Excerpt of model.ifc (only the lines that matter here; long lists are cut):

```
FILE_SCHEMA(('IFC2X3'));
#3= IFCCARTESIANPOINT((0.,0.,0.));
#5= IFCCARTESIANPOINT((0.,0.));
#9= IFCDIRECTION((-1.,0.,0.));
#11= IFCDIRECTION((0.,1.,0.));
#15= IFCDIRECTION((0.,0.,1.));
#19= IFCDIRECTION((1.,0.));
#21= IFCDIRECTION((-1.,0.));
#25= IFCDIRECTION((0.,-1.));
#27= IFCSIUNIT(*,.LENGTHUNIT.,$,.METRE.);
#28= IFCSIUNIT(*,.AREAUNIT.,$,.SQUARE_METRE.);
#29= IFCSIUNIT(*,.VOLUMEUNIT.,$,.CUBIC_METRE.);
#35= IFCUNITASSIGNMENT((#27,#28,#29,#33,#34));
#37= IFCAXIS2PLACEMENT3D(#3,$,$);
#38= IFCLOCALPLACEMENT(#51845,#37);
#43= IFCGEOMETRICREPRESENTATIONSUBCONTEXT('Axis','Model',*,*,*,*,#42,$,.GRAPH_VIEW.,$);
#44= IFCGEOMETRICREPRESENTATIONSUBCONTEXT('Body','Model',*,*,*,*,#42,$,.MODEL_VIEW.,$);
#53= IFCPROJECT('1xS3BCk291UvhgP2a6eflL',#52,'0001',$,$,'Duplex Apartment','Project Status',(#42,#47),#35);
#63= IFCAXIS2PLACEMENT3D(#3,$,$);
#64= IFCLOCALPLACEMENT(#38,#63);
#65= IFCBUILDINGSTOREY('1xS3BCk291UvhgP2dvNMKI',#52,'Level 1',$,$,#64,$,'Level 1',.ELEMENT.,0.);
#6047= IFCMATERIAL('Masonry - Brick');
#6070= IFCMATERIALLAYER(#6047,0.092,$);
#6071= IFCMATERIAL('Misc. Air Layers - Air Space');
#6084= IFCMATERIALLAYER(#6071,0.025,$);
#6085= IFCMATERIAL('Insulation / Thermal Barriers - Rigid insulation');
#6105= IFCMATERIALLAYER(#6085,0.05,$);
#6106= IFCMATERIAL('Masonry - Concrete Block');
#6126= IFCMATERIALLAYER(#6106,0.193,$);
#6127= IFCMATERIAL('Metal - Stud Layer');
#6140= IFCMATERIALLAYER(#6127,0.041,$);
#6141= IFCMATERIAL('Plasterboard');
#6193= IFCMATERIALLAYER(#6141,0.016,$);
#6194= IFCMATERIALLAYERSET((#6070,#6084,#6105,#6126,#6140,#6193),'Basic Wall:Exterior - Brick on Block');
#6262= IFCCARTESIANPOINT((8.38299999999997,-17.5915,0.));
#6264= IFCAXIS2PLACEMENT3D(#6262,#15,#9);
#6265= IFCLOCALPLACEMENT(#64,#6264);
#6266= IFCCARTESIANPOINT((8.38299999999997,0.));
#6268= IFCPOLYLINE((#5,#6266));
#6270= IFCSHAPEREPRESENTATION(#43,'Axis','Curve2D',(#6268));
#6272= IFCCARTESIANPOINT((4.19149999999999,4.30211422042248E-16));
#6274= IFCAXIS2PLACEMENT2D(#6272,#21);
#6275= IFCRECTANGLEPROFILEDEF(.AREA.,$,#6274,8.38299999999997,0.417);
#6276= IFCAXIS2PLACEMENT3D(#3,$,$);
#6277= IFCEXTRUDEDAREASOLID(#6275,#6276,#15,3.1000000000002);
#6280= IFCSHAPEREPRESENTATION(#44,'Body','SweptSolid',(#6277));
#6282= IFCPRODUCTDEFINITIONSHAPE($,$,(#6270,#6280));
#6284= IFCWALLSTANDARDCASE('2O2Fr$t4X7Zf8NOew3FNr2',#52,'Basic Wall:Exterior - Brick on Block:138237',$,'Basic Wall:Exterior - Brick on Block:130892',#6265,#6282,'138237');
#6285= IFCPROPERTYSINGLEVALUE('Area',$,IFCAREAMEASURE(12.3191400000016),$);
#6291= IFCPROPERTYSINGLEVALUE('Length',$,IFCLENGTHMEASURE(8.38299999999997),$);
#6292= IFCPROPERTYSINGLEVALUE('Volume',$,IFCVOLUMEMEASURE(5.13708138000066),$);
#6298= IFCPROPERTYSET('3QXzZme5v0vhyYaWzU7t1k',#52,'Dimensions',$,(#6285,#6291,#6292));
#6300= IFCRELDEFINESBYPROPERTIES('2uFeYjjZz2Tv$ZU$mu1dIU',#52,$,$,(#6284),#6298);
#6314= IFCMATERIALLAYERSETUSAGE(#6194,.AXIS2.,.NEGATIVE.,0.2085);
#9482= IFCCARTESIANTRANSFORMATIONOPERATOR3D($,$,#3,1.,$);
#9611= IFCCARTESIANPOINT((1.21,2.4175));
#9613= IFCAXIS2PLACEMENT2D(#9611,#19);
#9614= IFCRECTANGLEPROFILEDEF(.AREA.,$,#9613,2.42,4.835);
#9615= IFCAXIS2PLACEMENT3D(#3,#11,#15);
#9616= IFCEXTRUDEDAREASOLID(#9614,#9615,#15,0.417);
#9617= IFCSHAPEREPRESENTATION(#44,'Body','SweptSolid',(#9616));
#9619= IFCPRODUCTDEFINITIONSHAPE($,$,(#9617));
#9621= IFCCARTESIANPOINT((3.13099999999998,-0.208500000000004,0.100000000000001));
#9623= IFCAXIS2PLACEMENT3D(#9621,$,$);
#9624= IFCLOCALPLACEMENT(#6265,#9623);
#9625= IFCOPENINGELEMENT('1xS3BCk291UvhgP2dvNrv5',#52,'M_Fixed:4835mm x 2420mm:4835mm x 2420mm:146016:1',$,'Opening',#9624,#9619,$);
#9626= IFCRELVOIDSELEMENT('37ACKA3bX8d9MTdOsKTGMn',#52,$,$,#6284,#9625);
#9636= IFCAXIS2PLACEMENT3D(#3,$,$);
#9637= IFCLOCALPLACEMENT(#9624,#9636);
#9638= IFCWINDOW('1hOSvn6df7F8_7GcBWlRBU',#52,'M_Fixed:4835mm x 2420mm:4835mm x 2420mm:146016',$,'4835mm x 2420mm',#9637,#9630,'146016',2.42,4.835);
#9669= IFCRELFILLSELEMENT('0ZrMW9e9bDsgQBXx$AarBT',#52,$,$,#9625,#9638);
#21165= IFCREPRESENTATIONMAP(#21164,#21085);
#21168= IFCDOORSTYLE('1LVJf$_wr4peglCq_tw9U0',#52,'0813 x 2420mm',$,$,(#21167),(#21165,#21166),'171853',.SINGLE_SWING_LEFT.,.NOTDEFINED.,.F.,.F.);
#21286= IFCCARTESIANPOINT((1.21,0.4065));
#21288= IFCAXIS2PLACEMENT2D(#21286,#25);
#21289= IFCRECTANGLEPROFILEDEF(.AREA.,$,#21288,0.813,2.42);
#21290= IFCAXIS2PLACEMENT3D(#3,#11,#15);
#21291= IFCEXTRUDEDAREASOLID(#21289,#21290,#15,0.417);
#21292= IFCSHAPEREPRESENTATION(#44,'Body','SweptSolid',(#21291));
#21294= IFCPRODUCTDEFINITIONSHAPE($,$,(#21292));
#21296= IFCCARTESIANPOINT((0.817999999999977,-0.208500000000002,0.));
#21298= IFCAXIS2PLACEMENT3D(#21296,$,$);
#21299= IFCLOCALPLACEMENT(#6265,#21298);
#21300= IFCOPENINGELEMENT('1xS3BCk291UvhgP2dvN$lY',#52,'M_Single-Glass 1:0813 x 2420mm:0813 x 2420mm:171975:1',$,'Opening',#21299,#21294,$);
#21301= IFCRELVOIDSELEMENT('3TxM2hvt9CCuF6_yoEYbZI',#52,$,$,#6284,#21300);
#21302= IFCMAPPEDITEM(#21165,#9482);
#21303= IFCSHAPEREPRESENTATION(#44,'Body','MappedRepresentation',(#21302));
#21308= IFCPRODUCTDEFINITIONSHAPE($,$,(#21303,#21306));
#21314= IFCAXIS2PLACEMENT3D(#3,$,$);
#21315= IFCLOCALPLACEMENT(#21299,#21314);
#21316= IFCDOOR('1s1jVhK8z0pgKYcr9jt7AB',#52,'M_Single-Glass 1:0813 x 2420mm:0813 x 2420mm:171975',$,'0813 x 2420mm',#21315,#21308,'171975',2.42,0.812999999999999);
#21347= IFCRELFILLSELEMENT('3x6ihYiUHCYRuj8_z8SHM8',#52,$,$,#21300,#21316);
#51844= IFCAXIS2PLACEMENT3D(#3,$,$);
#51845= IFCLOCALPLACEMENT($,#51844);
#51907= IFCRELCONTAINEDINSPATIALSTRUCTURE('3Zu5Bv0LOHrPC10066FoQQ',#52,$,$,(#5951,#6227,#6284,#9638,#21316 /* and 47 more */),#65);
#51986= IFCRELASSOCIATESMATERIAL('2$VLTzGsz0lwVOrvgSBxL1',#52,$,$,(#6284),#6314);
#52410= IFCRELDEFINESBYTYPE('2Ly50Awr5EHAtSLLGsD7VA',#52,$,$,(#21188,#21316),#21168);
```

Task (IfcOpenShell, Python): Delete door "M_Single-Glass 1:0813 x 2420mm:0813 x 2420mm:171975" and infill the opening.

```python
import ifcopenshell
import ifcopenshell.api.feature
import ifcopenshell.api.pset
import ifcopenshell.api.root
import ifcopenshell.geom
import ifcopenshell.util.element
import ifcopenshell.util.shape
import ifcopenshell.util.unit

model = ifcopenshell.open("model.ifc")
area_scale = ifcopenshell.util.unit.calculate_unit_scale(model, "AREAUNIT")
volume_scale = ifcopenshell.util.unit.calculate_unit_scale(model, "VOLUMEUNIT")
settings = ifcopenshell.geom.settings()


def volume(element):
    """Net volume in cubic metres, openings subtracted."""
    shape = ifcopenshell.geom.create_shape(settings, element)
    return ifcopenshell.util.shape.get_volume(shape.geometry)


door = model.by_guid("1s1jVhK8z0pgKYcr9jt7AB")
opening = door.FillsVoids[0].RelatingOpeningElement
wall = opening.VoidsElements[0].RelatingBuildingElement
before = volume(wall)

ifcopenshell.api.root.remove_product(model, product=door)
ifcopenshell.api.feature.remove_feature(model, feature=opening)

after = volume(wall)
thickness = 0.417  # wall thickness in metres

# Update the wall's stored quantities.
pset = model.by_id(ifcopenshell.util.element.get_pset(wall, "Dimensions", should_inherit=False)["id"])
ifcopenshell.api.pset.edit_pset(model, pset=pset, properties={
    "Area": model.create_entity("IfcAreaMeasure", after / thickness / area_scale),
    "Volume": model.create_entity("IfcVolumeMeasure", after / volume_scale),
})

print(f"wall volume {before:.3f} -> {after:.3f} m3")

model.write("model_updated.ifc")
```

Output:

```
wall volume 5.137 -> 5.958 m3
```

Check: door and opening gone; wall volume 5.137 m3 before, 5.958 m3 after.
